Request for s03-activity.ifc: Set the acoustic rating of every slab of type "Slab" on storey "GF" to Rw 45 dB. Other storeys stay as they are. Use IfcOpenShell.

First a look at what the model holds.

```python
import ifcopenshell
import ifcopenshell.util.element

model = ifcopenshell.open("s03-activity.ifc")
print(model.schema)
storey = next(s for s in model.by_type("IfcBuildingStorey") if s.Name == "GF")
slabs = [e for e in ifcopenshell.util.element.get_decomposition(storey) if e.is_a("IfcSlab")]
seen = {}
for e in slabs:
    element_type = ifcopenshell.util.element.get_type(e)
    key = (element_type.Name if element_type != e and element_type else None, ifcopenshell.util.element.get_pset(e, "Pset_SlabCommon", "AcousticRating"))
    seen[key] = seen.get(key, 0) + 1
for (name, value), count in sorted(seen.items(), key=str):
    print(count, "x", name, "|", value)
```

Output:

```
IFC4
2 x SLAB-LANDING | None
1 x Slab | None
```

```python
import ifcopenshell
import ifcopenshell.api.pset
import ifcopenshell.util.element

model = ifcopenshell.open("s03-activity.ifc")

storey = next(s for s in model.by_type("IfcBuildingStorey") if s.Name == "GF")
slabs = [e for e in ifcopenshell.util.element.get_decomposition(storey) if e.is_a("IfcSlab")]

count = 0
for e in slabs:
    element_type = ifcopenshell.util.element.get_type(e)
    if element_type in (None, e) or element_type.Name != "Slab":
        continue
    # add_pset returns the element's existing set when there is one.
    pset = ifcopenshell.api.pset.add_pset(model, product=e, name="Pset_SlabCommon")
    ifcopenshell.api.pset.edit_pset(model, pset=pset, properties={"AcousticRating": "Rw 45 dB"})
    count += 1

print(count, "slabs updated")

model.write("s03-activity_v2.ifc")
```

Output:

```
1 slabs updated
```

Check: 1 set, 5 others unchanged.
